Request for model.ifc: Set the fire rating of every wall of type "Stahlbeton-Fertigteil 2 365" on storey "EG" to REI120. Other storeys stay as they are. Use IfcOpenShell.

First a look at what the model holds.

```python
import ifcopenshell
import ifcopenshell.util.element

model = ifcopenshell.open("model.ifc")
print(model.schema)
storey = next(s for s in model.by_type("IfcBuildingStorey") if s.Name == "EG")
walls = [e for e in ifcopenshell.util.element.get_decomposition(storey) if e.is_a("IfcWall")]
seen = {}
for e in walls:
    element_type = ifcopenshell.util.element.get_type(e)
    key = (element_type.Name if element_type != e and element_type else None, ifcopenshell.util.element.get_pset(e, "Pset_WallCommon", "FireRating"))
    seen[key] = seen.get(key, 0) + 1
for (name, value), count in sorted(seen.items(), key=str):
    print(count, "x", name, "|", value)
```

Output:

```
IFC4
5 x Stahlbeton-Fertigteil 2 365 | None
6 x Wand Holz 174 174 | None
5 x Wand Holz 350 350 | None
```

```python
import ifcopenshell
import ifcopenshell.api.pset
import ifcopenshell.util.element

model = ifcopenshell.open("model.ifc")

storey = next(s for s in model.by_type("IfcBuildingStorey") if s.Name == "EG")
walls = [e for e in ifcopenshell.util.element.get_decomposition(storey) if e.is_a("IfcWall")]

count = 0
for e in walls:
    element_type = ifcopenshell.util.element.get_type(e)
    if element_type in (None, e) or element_type.Name != "Stahlbeton-Fertigteil 2 365":
        continue
    # add_pset returns the element's existing set when there is one.
    pset = ifcopenshell.api.pset.add_pset(model, product=e, name="Pset_WallCommon")
    ifcopenshell.api.pset.edit_pset(model, pset=pset, properties={"FireRating": "REI120"})
    count += 1

print(count, "walls updated")

model.write("model_edited.ifc")
```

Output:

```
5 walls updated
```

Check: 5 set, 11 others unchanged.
